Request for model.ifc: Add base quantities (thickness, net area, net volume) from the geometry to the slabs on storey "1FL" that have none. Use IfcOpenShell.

First a look at what the model holds.

```python
import ifcopenshell
import ifcopenshell.util.element
import ifcopenshell.util.unit

model = ifcopenshell.open("model.ifc")
print(model.schema)
for unit_type in ("LENGTHUNIT", "AREAUNIT", "VOLUMEUNIT"):
    print(unit_type, ifcopenshell.util.unit.calculate_unit_scale(model, unit_type))
storey = next(s for s in model.by_type("IfcBuildingStorey") if s.Name == "1FL")
slabs = [e for e in ifcopenshell.util.element.get_decomposition(storey) if e.is_a("IfcSlab")]
for e in sorted(slabs, key=lambda e: e.id()):
    print(e.id(), e.is_a(), e.Name, list(ifcopenshell.util.element.get_psets(e, qtos_only=True)), sep=" | ")
```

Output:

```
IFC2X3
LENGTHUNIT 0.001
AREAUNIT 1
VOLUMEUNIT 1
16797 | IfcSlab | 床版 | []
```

```python
import ifcopenshell
import ifcopenshell.api.pset
import ifcopenshell.geom
import ifcopenshell.util.element
import ifcopenshell.util.shape
import ifcopenshell.util.unit

model = ifcopenshell.open("model.ifc")
unit_scale = ifcopenshell.util.unit.calculate_unit_scale(model)
area_scale = ifcopenshell.util.unit.calculate_unit_scale(model, "AREAUNIT")
volume_scale = ifcopenshell.util.unit.calculate_unit_scale(model, "VOLUMEUNIT")
settings = ifcopenshell.geom.settings()

storey = next(s for s in model.by_type("IfcBuildingStorey") if s.Name == "1FL")
slabs = [e for e in ifcopenshell.util.element.get_decomposition(storey) if e.is_a("IfcSlab")]

for e in sorted(slabs, key=lambda e: e.id()):
    if ifcopenshell.util.element.get_psets(e, qtos_only=True, should_inherit=False):
        continue
    # Geometry comes back in metres, in the element's own axes.
    shape = ifcopenshell.geom.create_shape(settings, e)
    values = {
        "Width": ifcopenshell.util.shape.get_z(shape.geometry) / unit_scale,
        "NetArea": ifcopenshell.util.shape.get_footprint_area(shape.geometry) / area_scale,
        "NetVolume": ifcopenshell.util.shape.get_volume(shape.geometry) / volume_scale,
    }
    qto = ifcopenshell.api.pset.add_qto(model, product=e, name="BaseQuantities")
    ifcopenshell.api.pset.edit_qto(model, qto=qto, properties=values)
    print(e.id(), {k: round(v, 3) for k, v in values.items()})

model.write("model-out.ifc")
```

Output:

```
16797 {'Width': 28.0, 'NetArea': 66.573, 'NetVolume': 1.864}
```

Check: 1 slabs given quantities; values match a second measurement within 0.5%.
